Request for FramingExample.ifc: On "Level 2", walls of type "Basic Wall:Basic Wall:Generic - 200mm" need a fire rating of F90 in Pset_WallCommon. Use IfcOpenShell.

First a look at what the model holds.

```python
import ifcopenshell
import ifcopenshell.util.element

model = ifcopenshell.open("FramingExample.ifc")
print(model.schema)
storey = next(s for s in model.by_type("IfcBuildingStorey") if s.Name == "Level 2")
walls = [e for e in ifcopenshell.util.element.get_decomposition(storey) if e.is_a("IfcWall")]
seen = {}
for e in walls:
    element_type = ifcopenshell.util.element.get_type(e)
    key = (element_type.Name if element_type != e and element_type else None, ifcopenshell.util.element.get_pset(e, "Pset_WallCommon", "FireRating"))
    seen[key] = seen.get(key, 0) + 1
for (name, value), count in sorted(seen.items(), key=str):
    print(count, "x", name, "|", value)
```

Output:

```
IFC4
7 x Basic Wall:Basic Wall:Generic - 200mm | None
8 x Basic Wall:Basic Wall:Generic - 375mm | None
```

```python
import ifcopenshell
import ifcopenshell.api.pset
import ifcopenshell.util.element

model = ifcopenshell.open("FramingExample.ifc")

storey = next(s for s in model.by_type("IfcBuildingStorey") if s.Name == "Level 2")
walls = [e for e in ifcopenshell.util.element.get_decomposition(storey) if e.is_a("IfcWall")]

count = 0
for e in walls:
    element_type = ifcopenshell.util.element.get_type(e)
    if element_type in (None, e) or element_type.Name != "Basic Wall:Basic Wall:Generic - 200mm":
        continue
    # add_pset returns the element's existing set when there is one.
    pset = ifcopenshell.api.pset.add_pset(model, product=e, name="Pset_WallCommon")
    ifcopenshell.api.pset.edit_pset(model, pset=pset, properties={"FireRating": "F90"})
    count += 1

print(count, "walls updated")

model.write("FramingExample_rev.ifc")
```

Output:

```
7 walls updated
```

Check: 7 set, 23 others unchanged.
